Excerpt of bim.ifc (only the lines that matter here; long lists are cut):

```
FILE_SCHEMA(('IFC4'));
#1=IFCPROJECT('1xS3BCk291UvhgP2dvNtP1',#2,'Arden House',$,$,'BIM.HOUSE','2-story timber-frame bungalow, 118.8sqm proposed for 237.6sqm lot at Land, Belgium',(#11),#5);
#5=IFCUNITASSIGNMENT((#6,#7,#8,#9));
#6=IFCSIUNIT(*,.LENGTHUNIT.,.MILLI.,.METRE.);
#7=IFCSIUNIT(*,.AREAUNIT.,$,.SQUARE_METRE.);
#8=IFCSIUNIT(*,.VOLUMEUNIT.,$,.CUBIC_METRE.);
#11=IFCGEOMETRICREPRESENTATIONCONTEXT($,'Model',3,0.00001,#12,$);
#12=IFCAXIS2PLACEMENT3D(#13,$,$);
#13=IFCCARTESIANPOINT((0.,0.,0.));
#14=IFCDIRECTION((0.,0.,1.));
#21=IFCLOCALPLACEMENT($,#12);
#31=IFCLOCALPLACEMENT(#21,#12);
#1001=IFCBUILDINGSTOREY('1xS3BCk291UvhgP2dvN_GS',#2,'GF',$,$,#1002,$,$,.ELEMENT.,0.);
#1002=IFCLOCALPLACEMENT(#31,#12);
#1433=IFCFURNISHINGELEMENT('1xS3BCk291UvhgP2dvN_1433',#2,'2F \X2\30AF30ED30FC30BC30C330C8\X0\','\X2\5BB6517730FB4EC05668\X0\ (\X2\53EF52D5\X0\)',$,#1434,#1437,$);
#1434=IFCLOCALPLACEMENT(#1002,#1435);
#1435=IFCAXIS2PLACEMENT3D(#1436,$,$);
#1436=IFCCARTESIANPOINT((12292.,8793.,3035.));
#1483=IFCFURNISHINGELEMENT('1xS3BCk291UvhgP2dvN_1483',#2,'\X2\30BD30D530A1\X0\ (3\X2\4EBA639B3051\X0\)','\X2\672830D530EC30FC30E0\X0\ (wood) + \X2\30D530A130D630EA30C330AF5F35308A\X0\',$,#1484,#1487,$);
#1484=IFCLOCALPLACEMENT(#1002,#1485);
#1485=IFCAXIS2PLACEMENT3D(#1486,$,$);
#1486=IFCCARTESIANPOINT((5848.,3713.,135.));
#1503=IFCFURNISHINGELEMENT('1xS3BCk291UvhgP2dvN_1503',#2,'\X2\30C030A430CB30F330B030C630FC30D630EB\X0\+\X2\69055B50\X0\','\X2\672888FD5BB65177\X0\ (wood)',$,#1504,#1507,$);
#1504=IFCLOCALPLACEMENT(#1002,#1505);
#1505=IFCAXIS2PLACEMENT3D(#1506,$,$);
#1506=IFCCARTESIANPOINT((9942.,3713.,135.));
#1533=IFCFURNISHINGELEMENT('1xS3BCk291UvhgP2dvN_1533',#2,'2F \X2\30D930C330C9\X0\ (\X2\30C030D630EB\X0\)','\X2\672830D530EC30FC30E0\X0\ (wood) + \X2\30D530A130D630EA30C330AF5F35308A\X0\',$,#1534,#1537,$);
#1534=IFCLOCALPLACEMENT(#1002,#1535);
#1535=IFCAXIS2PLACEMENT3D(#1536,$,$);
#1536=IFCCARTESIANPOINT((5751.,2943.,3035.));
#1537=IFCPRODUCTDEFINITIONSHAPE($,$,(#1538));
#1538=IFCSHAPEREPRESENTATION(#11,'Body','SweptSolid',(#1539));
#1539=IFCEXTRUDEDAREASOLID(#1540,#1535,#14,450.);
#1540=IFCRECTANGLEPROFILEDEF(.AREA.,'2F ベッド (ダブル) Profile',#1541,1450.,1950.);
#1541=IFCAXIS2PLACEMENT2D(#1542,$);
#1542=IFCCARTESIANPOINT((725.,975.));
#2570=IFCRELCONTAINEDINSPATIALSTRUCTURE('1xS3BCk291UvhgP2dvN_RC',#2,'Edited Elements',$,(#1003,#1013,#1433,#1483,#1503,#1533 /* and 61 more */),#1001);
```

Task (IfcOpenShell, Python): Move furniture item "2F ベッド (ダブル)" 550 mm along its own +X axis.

```python
import ifcopenshell
import ifcopenshell.api.geometry
import ifcopenshell.util.placement

model = ifcopenshell.open("bim.ifc")

item = model.by_guid("1xS3BCk291UvhgP2dvN_1533")
matrix = ifcopenshell.util.placement.get_local_placement(item.ObjectPlacement)
matrix[:3, 3] += matrix[:3, 0] * 550.0
ifcopenshell.api.geometry.edit_object_placement(model, product=item, matrix=matrix, is_si=False)

print(ifcopenshell.util.placement.get_local_placement(item.ObjectPlacement).round(3) + 0.0)

model.write("bim-out.ifc")
```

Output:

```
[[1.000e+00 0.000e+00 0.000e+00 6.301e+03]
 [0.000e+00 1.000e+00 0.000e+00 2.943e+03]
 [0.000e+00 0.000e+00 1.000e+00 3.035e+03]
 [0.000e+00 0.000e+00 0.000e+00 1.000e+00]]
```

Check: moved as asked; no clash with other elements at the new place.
